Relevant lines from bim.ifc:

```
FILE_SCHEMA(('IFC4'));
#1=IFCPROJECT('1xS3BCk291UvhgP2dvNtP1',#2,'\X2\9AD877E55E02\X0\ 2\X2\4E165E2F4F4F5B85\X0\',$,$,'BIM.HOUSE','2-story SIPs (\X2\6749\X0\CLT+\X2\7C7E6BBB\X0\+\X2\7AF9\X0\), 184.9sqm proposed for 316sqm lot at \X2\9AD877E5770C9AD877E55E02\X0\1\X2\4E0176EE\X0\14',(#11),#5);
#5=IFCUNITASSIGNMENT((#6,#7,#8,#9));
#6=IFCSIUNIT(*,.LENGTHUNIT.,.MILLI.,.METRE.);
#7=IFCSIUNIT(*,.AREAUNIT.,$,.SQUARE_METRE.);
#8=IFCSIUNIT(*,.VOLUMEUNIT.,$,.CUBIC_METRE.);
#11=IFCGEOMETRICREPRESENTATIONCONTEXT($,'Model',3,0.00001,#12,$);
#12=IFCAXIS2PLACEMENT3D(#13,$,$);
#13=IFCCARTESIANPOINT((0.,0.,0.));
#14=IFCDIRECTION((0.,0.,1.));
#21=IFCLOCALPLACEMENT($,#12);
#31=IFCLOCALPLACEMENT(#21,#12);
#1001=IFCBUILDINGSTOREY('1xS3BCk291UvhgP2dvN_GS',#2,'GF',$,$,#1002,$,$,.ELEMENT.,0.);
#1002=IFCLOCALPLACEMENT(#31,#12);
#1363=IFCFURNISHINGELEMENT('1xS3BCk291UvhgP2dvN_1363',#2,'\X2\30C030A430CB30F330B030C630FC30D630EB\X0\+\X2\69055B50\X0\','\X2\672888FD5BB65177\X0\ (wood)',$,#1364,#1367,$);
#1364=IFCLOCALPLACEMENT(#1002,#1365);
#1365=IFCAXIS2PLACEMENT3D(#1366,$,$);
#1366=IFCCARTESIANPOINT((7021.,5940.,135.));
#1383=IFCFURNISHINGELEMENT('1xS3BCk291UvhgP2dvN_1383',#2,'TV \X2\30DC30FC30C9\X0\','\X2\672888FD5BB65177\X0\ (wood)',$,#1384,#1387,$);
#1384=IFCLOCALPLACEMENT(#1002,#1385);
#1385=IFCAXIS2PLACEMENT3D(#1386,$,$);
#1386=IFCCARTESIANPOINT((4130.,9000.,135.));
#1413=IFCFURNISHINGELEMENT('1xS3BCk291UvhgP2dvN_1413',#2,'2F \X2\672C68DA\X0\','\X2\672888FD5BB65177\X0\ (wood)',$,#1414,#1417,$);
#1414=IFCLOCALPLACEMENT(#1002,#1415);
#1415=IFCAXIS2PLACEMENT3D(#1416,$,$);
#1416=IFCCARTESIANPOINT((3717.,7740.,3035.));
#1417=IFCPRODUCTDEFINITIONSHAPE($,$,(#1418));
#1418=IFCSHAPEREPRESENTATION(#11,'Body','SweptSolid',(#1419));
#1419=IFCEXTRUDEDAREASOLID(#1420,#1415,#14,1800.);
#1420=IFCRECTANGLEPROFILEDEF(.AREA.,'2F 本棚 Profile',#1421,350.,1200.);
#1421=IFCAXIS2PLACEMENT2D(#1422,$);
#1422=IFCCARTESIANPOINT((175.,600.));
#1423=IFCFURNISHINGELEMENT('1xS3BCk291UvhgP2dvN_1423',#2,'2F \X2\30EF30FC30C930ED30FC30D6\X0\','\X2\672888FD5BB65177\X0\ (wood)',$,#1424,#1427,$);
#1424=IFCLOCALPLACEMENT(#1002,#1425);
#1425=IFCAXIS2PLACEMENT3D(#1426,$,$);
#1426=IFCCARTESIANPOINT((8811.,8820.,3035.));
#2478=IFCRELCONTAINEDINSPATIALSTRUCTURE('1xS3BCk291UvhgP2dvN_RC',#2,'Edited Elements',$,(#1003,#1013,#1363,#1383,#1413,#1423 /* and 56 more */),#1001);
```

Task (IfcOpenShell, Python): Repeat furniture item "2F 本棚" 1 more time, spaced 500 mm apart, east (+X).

```python
import numpy as np
import ifcopenshell
import ifcopenshell.api.geometry
import ifcopenshell.api.root
import ifcopenshell.util.element
import ifcopenshell.util.placement
import ifcopenshell.util.unit

model = ifcopenshell.open("bim.ifc")
unit_scale = ifcopenshell.util.unit.calculate_unit_scale(model)


def reuse_history(source, copy):
    """copy_class also copies each property set's owner history, people and application; keep the originals."""
    for rel in copy.IsDefinedBy:
        if rel.is_a("IfcRelDefinesByProperties") and (history := rel.RelatingPropertyDefinition.OwnerHistory):
            rel.RelatingPropertyDefinition.OwnerHistory = source.OwnerHistory
            ifcopenshell.util.element.remove_deep2(model, history)


source = model.by_guid("1xS3BCk291UvhgP2dvN_1413")
base = ifcopenshell.util.placement.get_local_placement(source.ObjectPlacement)
step = np.array([1.0, 0.0, 0.0]) * 0.5 / unit_scale

for i in range(1, 2):
    copy = ifcopenshell.api.root.copy_class(model, product=source)
    copy.Representation = ifcopenshell.util.element.copy_deep(
        model, source.Representation, exclude=["IfcGeometricRepresentationContext", "IfcRepresentationMap"]
    )
    reuse_history(source, copy)
    matrix = base.copy()
    matrix[:3, 3] += i * step
    print("added at", matrix[:3, 3].round(3) + 0.0)
    ifcopenshell.api.geometry.edit_object_placement(model, product=copy, matrix=matrix, is_si=False)

model.write("bim_v2.ifc")
```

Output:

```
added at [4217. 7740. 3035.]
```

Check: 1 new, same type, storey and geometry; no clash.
